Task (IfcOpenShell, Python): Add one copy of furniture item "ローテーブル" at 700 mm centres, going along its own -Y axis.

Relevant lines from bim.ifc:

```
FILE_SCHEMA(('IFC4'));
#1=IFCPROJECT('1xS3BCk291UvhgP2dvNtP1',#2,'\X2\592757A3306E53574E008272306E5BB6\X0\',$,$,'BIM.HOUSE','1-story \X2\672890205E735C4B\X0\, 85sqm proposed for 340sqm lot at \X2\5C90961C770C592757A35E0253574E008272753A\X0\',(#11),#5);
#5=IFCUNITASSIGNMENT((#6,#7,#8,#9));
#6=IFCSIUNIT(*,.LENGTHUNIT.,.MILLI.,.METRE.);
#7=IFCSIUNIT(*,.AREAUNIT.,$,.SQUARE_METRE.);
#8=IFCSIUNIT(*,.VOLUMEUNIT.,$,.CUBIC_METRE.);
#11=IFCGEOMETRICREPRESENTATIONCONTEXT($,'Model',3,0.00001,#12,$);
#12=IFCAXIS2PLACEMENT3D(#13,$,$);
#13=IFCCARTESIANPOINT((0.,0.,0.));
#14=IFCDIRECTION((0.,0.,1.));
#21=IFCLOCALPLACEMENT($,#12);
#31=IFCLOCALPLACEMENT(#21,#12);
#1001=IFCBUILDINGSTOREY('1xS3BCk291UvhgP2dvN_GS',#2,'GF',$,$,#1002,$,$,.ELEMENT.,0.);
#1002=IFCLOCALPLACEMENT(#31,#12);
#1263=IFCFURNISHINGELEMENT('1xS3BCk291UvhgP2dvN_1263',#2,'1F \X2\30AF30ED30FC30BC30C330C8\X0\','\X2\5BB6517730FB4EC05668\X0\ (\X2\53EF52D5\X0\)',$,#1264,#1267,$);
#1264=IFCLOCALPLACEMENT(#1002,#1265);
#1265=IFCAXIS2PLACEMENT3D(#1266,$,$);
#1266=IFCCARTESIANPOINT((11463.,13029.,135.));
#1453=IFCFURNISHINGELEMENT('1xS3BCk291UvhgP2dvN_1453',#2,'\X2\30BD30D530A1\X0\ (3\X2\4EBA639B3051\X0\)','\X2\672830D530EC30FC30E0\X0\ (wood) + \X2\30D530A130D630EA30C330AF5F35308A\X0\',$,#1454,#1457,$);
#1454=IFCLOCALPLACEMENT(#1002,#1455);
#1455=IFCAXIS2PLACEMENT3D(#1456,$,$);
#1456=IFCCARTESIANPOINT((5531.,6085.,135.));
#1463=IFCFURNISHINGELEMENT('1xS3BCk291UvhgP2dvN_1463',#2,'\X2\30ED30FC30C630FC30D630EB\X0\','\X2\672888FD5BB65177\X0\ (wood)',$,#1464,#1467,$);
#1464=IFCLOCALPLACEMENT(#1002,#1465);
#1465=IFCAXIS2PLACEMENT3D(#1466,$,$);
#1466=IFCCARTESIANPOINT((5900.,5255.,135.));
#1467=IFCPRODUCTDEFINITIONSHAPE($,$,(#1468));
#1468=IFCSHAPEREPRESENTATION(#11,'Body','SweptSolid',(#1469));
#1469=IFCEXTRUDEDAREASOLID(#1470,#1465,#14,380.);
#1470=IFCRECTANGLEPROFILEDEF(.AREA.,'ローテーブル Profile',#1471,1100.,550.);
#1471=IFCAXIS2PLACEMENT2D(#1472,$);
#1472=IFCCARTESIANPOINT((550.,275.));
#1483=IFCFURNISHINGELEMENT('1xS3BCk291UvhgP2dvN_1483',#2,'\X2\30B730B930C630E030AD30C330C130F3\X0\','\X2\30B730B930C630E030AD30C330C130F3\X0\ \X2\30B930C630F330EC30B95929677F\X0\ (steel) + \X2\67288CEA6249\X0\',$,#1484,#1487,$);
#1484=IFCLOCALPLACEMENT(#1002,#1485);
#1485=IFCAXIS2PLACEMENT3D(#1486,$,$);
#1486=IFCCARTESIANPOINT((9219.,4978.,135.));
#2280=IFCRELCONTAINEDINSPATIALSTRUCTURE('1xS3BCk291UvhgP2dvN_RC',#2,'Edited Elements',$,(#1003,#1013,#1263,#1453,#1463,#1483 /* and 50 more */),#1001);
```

```python
import ifcopenshell
import ifcopenshell.api.geometry
import ifcopenshell.api.root
import ifcopenshell.util.element
import ifcopenshell.util.placement

model = ifcopenshell.open("bim.ifc")


def reuse_history(source, copy):
    """copy_class also copies each property set's owner history, people and application; keep the originals."""
    for rel in copy.IsDefinedBy:
        if rel.is_a("IfcRelDefinesByProperties") and (history := rel.RelatingPropertyDefinition.OwnerHistory):
            rel.RelatingPropertyDefinition.OwnerHistory = source.OwnerHistory
            ifcopenshell.util.element.remove_deep2(model, history)


source = model.by_guid("1xS3BCk291UvhgP2dvN_1463")
base = ifcopenshell.util.placement.get_local_placement(source.ObjectPlacement)
step = -base[:3, 1] * 700.0

for i in range(1, 2):
    copy = ifcopenshell.api.root.copy_class(model, product=source)
    copy.Representation = ifcopenshell.util.element.copy_deep(
        model, source.Representation, exclude=["IfcGeometricRepresentationContext", "IfcRepresentationMap"]
    )
    reuse_history(source, copy)
    matrix = base.copy()
    matrix[:3, 3] += i * step
    print("added at", matrix[:3, 3].round(3) + 0.0)
    ifcopenshell.api.geometry.edit_object_placement(model, product=copy, matrix=matrix, is_si=False)

model.write("bim_updated.ifc")
```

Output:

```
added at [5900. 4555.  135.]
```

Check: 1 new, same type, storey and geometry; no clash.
